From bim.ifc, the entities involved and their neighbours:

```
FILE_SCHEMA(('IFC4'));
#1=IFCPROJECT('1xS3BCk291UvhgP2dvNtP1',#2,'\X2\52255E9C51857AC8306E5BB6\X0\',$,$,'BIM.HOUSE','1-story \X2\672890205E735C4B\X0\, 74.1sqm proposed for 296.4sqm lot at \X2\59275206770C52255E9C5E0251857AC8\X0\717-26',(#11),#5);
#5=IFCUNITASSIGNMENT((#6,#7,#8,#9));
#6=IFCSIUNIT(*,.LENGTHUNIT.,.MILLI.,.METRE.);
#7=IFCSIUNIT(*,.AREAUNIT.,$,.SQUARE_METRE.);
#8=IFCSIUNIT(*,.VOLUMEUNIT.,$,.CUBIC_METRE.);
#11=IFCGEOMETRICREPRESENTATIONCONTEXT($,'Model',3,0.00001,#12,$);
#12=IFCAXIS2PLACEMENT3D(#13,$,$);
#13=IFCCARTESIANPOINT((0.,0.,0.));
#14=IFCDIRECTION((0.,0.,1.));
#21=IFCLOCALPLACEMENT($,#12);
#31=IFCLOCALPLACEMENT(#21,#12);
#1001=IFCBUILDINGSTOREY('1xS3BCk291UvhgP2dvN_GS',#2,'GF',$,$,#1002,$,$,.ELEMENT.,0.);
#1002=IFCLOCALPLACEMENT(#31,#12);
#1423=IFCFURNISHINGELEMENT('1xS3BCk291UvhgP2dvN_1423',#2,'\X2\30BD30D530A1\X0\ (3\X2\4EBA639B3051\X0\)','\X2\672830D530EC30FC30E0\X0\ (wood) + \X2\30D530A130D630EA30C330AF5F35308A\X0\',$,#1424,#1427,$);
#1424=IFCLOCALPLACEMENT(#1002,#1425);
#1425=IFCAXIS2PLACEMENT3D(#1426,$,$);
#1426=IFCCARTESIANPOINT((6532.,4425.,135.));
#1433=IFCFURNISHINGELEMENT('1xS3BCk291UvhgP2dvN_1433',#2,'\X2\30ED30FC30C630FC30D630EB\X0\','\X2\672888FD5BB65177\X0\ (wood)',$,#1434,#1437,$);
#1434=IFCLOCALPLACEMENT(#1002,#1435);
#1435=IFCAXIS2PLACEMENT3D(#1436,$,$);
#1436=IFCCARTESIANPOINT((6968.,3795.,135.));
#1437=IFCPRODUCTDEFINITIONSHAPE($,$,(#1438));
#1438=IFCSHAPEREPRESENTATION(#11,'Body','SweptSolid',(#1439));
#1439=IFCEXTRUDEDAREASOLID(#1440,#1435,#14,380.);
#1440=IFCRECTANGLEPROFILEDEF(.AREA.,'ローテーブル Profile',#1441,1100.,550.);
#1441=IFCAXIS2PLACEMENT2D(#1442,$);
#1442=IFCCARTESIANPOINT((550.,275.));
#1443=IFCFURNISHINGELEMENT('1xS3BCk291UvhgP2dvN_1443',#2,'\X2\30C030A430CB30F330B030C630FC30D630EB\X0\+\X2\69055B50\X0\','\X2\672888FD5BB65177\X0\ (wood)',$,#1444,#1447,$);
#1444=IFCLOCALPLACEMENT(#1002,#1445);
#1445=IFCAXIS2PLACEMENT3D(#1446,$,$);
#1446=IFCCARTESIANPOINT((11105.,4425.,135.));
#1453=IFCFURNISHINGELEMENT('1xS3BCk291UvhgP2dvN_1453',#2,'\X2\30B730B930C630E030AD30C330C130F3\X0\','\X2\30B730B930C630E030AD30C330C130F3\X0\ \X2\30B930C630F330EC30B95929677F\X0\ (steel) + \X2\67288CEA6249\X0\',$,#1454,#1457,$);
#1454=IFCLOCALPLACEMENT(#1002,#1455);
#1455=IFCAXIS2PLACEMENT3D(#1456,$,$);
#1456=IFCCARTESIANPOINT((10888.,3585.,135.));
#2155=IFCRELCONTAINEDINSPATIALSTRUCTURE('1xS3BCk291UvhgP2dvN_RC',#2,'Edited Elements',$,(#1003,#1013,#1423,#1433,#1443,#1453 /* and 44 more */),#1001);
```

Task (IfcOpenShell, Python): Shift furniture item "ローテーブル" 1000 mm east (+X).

```python
import ifcopenshell
import ifcopenshell.api.geometry
import ifcopenshell.util.placement

model = ifcopenshell.open("bim.ifc")

item = model.by_guid("1xS3BCk291UvhgP2dvN_1433")
matrix = ifcopenshell.util.placement.get_local_placement(item.ObjectPlacement)
matrix[0, 3] += 1000.0
ifcopenshell.api.geometry.edit_object_placement(model, product=item, matrix=matrix, is_si=False)

print(ifcopenshell.util.placement.get_local_placement(item.ObjectPlacement).round(3) + 0.0)

model.write("bim-out.ifc")
```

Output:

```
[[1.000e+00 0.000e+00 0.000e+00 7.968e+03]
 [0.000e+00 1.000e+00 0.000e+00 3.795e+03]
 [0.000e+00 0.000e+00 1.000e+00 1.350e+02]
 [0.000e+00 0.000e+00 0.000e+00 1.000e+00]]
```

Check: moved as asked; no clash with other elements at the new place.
